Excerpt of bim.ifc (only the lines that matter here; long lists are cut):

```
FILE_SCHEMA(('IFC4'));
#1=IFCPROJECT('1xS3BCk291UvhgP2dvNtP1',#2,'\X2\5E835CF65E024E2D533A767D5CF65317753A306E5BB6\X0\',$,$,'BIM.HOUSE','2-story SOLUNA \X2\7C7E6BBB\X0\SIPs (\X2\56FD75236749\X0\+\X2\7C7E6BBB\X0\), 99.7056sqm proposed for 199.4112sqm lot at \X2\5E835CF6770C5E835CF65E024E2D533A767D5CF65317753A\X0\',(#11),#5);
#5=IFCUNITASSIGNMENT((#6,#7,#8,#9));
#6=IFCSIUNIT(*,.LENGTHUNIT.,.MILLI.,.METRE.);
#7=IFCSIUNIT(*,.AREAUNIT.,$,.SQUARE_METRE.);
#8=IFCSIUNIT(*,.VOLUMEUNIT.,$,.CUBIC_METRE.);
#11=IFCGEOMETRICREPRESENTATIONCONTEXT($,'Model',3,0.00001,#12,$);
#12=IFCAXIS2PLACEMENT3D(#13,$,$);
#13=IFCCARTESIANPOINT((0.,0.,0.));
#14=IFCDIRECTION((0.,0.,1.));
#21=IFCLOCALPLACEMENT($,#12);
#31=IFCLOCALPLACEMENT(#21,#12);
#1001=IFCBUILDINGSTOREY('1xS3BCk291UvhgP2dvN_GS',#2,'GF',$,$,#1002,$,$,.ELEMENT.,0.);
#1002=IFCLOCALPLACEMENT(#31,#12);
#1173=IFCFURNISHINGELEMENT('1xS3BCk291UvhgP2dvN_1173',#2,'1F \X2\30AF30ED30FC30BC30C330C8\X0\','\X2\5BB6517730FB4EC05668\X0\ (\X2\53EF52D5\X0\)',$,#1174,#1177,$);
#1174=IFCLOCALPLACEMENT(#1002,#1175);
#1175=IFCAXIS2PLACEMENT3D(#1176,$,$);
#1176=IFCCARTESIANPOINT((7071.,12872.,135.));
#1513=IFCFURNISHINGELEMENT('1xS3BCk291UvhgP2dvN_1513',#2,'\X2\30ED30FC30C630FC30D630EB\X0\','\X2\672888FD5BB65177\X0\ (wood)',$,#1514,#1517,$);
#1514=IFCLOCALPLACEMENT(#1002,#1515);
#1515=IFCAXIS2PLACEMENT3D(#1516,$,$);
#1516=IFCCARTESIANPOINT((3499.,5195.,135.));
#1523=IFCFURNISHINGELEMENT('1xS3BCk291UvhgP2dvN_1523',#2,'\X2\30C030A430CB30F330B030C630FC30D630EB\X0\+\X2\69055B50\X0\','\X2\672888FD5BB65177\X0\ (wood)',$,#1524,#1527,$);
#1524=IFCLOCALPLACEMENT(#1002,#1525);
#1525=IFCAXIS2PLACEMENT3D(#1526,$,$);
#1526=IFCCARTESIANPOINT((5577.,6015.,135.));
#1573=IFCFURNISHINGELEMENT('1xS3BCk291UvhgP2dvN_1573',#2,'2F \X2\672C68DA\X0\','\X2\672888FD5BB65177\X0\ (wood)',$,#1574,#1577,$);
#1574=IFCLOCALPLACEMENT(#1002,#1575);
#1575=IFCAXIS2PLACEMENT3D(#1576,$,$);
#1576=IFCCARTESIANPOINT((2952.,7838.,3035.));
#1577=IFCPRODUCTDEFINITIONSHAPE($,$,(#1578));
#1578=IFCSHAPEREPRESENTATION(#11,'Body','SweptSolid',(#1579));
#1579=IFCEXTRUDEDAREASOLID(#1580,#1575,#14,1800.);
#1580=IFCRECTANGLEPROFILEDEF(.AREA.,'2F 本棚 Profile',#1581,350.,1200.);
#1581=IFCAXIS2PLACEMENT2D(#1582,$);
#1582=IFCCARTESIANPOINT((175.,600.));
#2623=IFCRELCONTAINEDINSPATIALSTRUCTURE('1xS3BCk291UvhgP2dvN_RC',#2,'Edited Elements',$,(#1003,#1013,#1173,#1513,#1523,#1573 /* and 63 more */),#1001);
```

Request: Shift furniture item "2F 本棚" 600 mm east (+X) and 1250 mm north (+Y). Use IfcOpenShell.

```python
import ifcopenshell
import ifcopenshell.api.geometry
import ifcopenshell.util.placement
import ifcopenshell.util.unit

model = ifcopenshell.open("bim.ifc")
unit_scale = ifcopenshell.util.unit.calculate_unit_scale(model)

item = model.by_guid("1xS3BCk291UvhgP2dvN_1573")
matrix = ifcopenshell.util.placement.get_local_placement(item.ObjectPlacement)
matrix[0, 3] += 0.6 / unit_scale
matrix[1, 3] += 1.25 / unit_scale
ifcopenshell.api.geometry.edit_object_placement(model, product=item, matrix=matrix, is_si=False)

print(ifcopenshell.util.placement.get_local_placement(item.ObjectPlacement).round(3) + 0.0)

model.write("bim_v2.ifc")
```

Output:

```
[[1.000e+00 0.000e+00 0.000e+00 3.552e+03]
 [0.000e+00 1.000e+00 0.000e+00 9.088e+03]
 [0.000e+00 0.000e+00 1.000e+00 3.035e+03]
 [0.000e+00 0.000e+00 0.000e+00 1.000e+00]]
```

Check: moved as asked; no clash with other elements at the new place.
